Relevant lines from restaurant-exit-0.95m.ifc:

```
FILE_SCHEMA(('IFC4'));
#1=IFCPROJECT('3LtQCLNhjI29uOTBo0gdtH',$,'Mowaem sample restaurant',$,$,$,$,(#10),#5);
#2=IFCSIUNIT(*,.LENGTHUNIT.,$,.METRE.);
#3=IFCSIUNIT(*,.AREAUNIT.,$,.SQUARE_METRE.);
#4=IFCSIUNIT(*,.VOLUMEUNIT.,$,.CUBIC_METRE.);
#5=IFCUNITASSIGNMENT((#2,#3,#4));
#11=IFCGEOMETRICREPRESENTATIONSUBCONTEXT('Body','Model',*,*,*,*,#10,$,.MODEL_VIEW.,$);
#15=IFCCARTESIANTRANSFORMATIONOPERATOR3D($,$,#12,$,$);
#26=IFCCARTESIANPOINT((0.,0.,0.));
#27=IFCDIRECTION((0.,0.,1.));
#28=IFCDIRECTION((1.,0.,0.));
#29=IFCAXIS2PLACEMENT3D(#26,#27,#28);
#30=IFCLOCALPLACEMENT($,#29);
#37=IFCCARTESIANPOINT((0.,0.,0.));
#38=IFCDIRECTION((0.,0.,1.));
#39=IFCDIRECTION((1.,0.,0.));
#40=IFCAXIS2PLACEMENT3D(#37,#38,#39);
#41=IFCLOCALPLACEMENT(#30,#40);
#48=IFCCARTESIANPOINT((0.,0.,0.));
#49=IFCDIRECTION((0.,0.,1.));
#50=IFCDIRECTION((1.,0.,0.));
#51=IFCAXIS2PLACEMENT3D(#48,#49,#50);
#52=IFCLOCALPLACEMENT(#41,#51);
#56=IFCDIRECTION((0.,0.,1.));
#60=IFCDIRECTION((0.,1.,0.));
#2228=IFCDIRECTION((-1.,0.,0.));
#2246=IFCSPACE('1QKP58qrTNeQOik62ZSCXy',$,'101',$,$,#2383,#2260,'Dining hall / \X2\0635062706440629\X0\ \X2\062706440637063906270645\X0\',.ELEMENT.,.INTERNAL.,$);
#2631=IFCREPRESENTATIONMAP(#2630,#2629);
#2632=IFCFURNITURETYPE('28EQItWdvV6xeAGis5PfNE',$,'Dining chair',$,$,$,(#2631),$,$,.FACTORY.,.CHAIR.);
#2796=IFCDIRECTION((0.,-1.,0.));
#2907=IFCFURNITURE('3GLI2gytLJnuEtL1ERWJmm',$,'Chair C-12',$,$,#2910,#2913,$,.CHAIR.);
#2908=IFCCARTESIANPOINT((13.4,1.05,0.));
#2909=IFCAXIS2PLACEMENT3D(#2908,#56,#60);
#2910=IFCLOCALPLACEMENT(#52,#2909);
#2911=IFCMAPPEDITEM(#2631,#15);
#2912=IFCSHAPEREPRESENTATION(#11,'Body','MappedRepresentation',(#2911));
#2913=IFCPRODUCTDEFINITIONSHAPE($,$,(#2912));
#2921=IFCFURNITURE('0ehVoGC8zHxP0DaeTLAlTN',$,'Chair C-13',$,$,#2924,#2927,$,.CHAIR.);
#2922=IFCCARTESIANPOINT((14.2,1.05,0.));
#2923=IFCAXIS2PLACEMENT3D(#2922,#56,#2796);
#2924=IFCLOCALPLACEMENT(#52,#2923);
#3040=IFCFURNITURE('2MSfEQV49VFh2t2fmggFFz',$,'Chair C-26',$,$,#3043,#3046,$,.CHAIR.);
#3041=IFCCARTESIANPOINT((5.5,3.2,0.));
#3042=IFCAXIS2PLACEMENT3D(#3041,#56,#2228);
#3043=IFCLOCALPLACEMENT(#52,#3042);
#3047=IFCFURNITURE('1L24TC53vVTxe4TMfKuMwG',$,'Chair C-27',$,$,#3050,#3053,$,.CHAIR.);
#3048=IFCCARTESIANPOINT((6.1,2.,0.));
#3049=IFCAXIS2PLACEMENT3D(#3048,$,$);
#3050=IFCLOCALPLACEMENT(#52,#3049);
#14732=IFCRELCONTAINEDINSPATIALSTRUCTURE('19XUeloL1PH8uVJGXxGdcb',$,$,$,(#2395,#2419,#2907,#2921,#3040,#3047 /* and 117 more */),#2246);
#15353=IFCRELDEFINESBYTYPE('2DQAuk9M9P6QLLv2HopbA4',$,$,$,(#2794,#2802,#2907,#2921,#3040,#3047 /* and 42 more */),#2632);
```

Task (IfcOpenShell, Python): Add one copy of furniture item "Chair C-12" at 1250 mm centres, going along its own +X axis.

```python
import ifcopenshell
import ifcopenshell.api.geometry
import ifcopenshell.api.root
import ifcopenshell.util.element
import ifcopenshell.util.placement

model = ifcopenshell.open("restaurant-exit-0.95m.ifc")

source = model.by_guid("3GLI2gytLJnuEtL1ERWJmm")
base = ifcopenshell.util.placement.get_local_placement(source.ObjectPlacement)
step = base[:3, 0] * 1.25

for i in range(1, 2):
    copy = ifcopenshell.api.root.copy_class(model, product=source)
    copy.Representation = ifcopenshell.util.element.copy_deep(
        model, source.Representation, exclude=["IfcGeometricRepresentationContext", "IfcRepresentationMap"]
    )
    matrix = base.copy()
    matrix[:3, 3] += i * step
    print("added at", matrix[:3, 3].round(3) + 0.0)
    ifcopenshell.api.geometry.edit_object_placement(model, product=copy, matrix=matrix, is_si=False)

model.write("restaurant-exit-0.95m_edited.ifc")
```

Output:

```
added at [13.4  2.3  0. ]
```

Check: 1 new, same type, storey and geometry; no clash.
